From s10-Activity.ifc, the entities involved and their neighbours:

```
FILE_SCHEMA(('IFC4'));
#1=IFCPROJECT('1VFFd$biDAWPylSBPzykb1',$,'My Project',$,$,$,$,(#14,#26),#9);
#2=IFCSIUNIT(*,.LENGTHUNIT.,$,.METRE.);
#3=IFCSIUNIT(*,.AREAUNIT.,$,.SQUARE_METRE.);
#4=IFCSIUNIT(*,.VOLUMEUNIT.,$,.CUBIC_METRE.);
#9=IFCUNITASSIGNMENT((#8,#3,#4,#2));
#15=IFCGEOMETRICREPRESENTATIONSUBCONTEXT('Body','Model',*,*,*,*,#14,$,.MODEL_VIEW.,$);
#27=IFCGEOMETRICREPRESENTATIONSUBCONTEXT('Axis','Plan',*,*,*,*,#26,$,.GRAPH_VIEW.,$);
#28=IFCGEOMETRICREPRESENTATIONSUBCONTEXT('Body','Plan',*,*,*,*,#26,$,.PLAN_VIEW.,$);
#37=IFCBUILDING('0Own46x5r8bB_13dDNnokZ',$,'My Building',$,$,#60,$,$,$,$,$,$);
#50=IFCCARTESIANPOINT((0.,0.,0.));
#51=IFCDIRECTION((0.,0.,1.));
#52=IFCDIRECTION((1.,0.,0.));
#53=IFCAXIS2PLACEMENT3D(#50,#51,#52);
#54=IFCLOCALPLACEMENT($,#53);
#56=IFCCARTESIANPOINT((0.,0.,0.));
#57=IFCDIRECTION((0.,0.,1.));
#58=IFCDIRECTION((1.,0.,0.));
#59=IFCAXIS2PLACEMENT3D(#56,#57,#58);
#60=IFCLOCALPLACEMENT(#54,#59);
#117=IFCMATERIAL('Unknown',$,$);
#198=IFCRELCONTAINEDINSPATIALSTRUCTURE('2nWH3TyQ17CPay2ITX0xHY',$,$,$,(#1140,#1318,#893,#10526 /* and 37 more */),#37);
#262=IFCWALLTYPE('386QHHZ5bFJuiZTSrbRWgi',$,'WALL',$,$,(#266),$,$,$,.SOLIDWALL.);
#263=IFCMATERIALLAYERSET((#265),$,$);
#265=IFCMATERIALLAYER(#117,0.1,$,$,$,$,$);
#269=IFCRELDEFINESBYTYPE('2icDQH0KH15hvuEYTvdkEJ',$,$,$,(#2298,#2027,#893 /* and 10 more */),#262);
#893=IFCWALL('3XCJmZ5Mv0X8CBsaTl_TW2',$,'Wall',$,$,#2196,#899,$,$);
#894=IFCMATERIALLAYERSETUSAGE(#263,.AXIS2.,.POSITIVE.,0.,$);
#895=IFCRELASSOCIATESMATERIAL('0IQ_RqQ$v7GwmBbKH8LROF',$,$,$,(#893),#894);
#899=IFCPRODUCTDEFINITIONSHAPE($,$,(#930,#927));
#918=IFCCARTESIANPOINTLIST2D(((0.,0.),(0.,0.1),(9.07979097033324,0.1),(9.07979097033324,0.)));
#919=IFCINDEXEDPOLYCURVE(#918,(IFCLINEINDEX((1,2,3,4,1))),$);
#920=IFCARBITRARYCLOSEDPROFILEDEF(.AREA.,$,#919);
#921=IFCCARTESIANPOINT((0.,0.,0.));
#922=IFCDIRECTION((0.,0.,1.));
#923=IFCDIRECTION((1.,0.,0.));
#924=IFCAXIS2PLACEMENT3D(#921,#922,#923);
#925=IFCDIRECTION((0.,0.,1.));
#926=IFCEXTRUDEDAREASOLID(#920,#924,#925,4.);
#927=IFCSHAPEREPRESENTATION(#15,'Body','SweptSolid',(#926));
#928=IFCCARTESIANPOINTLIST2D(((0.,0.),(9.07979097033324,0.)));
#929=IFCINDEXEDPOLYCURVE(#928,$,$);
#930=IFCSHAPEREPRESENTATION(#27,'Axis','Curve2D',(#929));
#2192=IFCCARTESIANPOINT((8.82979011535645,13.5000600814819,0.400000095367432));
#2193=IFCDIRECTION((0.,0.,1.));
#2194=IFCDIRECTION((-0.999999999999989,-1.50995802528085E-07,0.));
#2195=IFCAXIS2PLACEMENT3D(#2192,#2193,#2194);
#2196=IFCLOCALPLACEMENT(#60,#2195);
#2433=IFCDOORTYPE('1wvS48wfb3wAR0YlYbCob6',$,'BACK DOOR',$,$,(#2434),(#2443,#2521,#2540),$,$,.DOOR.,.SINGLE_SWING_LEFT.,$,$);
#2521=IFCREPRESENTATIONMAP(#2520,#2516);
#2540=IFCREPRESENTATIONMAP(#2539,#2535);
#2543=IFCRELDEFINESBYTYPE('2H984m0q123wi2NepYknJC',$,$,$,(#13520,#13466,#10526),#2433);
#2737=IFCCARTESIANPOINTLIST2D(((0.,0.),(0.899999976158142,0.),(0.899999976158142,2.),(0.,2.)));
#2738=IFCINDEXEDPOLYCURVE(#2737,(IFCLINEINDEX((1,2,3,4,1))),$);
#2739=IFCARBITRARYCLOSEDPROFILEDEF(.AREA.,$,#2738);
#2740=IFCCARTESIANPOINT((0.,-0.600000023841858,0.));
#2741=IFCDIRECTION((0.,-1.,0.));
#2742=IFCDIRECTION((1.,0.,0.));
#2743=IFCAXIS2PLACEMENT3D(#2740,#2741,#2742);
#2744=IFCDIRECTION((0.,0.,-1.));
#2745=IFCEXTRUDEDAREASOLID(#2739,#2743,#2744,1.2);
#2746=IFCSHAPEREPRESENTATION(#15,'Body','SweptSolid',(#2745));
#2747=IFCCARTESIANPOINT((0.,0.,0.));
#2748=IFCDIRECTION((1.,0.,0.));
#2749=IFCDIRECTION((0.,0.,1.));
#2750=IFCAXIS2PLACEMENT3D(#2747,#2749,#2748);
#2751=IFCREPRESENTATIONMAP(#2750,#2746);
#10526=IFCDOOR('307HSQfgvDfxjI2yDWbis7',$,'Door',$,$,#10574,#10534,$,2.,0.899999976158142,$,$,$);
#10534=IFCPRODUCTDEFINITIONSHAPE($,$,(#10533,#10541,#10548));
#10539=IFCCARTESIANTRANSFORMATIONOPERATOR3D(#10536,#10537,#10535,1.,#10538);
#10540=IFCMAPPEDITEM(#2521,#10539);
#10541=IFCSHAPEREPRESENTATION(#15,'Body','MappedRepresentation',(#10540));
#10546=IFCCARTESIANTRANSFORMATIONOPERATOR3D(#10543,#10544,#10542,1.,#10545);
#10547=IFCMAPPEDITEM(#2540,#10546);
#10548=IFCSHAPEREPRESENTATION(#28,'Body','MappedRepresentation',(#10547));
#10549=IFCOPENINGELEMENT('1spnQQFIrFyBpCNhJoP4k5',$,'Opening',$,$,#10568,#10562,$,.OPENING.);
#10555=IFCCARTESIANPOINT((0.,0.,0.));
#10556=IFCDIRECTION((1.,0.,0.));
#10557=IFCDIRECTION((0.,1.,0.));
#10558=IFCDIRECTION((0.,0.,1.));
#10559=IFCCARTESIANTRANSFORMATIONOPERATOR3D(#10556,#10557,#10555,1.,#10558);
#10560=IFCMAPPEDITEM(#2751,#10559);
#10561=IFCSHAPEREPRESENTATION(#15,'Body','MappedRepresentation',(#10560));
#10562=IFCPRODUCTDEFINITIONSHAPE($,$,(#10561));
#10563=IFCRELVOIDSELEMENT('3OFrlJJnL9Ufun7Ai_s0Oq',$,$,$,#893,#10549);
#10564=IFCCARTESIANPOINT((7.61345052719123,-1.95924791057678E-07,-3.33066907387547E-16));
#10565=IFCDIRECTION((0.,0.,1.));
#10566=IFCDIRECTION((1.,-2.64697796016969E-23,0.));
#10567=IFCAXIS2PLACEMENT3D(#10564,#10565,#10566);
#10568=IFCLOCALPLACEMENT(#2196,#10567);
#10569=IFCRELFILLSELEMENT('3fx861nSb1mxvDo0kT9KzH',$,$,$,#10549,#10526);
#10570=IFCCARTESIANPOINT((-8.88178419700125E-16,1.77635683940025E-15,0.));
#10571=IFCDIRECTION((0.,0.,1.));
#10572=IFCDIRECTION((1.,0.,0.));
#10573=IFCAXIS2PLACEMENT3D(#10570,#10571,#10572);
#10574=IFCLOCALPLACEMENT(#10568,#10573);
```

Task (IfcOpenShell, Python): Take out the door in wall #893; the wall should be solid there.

```python
import ifcopenshell
import ifcopenshell.api.feature
import ifcopenshell.api.root
import ifcopenshell.geom
import ifcopenshell.util.shape

model = ifcopenshell.open("s10-Activity.ifc")
settings = ifcopenshell.geom.settings()


def volume(element):
    """Net volume in cubic metres, openings subtracted."""
    shape = ifcopenshell.geom.create_shape(settings, element)
    return ifcopenshell.util.shape.get_volume(shape.geometry)


door = model.by_guid("307HSQfgvDfxjI2yDWbis7")
opening = door.FillsVoids[0].RelatingOpeningElement
wall = opening.VoidsElements[0].RelatingBuildingElement
before = volume(wall)

ifcopenshell.api.root.remove_product(model, product=door)
ifcopenshell.api.feature.remove_feature(model, feature=opening)

after = volume(wall)

print(f"wall volume {before:.3f} -> {after:.3f} m3")

model.write("s10-Activity_rev.ifc")
```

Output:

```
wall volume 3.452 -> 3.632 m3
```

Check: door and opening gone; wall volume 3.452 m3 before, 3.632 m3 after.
